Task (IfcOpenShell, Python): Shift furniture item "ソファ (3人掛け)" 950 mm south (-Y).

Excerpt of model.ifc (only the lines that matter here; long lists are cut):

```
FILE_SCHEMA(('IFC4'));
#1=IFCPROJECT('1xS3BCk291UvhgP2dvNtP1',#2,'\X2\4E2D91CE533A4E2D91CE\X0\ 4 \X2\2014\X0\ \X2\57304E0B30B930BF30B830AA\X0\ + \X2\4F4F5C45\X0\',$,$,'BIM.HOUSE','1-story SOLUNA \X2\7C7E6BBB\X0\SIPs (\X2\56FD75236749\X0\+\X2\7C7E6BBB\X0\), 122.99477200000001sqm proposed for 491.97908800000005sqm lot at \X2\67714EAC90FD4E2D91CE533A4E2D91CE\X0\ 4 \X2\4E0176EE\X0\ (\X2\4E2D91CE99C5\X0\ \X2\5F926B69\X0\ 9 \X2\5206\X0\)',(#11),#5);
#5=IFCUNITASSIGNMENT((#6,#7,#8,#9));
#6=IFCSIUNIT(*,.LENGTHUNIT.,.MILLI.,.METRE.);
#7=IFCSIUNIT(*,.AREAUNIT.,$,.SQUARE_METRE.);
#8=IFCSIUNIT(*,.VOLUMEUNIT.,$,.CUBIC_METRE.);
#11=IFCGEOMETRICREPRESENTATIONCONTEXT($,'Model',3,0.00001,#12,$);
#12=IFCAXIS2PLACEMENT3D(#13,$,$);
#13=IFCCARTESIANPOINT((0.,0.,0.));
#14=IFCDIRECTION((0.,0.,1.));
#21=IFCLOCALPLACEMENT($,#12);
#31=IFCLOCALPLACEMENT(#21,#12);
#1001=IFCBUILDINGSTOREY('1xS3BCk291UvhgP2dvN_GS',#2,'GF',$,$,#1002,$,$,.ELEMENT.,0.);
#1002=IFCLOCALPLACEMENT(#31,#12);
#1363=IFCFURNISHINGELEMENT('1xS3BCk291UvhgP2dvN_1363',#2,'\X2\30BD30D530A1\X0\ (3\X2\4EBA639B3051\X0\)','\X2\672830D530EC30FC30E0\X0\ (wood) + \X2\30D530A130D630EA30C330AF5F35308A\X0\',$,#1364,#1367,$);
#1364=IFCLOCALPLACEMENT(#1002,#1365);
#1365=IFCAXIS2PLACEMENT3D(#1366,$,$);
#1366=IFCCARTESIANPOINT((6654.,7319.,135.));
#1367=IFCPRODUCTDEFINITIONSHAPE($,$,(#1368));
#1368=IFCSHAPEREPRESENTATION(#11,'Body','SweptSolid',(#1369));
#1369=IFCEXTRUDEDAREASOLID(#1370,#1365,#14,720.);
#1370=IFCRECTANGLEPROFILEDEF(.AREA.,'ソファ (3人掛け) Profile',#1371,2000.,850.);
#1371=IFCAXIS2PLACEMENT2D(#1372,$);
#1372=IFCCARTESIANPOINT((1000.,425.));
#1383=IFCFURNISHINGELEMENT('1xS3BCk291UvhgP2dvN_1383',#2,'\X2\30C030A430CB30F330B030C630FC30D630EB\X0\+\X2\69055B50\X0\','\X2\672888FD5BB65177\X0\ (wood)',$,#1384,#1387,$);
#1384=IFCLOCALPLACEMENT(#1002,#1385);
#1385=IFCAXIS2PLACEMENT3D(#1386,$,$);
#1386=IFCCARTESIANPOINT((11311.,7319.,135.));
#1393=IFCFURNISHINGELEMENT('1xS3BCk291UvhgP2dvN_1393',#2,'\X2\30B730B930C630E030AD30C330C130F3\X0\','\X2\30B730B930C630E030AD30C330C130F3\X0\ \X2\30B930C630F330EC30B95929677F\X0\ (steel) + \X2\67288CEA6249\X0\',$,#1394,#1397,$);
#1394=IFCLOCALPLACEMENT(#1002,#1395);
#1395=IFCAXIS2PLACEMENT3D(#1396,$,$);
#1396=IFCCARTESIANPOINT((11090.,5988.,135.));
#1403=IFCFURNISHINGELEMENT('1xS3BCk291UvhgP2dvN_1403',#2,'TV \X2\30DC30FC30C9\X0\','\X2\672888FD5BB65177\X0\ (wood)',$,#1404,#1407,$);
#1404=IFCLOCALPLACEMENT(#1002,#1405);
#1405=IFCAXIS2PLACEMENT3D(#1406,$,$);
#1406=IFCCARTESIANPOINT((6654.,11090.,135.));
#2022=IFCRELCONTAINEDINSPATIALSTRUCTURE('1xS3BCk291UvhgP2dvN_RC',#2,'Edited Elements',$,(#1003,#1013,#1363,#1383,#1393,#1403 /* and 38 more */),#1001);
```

```python
import ifcopenshell
import ifcopenshell.api.geometry
import ifcopenshell.util.placement

model = ifcopenshell.open("model.ifc")

item = model.by_guid("1xS3BCk291UvhgP2dvN_1363")
matrix = ifcopenshell.util.placement.get_local_placement(item.ObjectPlacement)
matrix[1, 3] -= 950.0
ifcopenshell.api.geometry.edit_object_placement(model, product=item, matrix=matrix, is_si=False)

print(ifcopenshell.util.placement.get_local_placement(item.ObjectPlacement).round(3) + 0.0)

model.write("model_rev.ifc")
```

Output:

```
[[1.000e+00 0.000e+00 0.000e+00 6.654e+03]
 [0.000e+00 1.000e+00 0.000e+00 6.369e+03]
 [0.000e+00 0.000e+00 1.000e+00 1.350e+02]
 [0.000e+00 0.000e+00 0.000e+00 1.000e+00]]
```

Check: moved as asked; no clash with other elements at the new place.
